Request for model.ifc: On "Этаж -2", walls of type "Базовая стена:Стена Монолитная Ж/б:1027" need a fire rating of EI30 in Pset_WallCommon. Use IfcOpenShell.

First a look at what the model holds.

```python
import ifcopenshell
import ifcopenshell.util.element

model = ifcopenshell.open("model.ifc")
print(model.schema)
storey = next(s for s in model.by_type("IfcBuildingStorey") if s.Name == "Этаж -2")
walls = [e for e in ifcopenshell.util.element.get_decomposition(storey) if e.is_a("IfcWall")]
seen = {}
for e in walls:
    element_type = ifcopenshell.util.element.get_type(e)
    key = (element_type.Name if element_type != e and element_type else None, ifcopenshell.util.element.get_pset(e, "Pset_WallCommon", "FireRating"))
    seen[key] = seen.get(key, 0) + 1
for (name, value), count in sorted(seen.items(), key=str):
    print(count, "x", name, "|", value)
```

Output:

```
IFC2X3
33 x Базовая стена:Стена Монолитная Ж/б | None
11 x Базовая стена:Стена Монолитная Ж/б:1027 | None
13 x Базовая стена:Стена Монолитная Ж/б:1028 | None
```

```python
import ifcopenshell
import ifcopenshell.api.pset
import ifcopenshell.util.element

model = ifcopenshell.open("model.ifc")

storey = next(s for s in model.by_type("IfcBuildingStorey") if s.Name == "Этаж -2")
walls = [e for e in ifcopenshell.util.element.get_decomposition(storey) if e.is_a("IfcWall")]

count = 0
for e in walls:
    element_type = ifcopenshell.util.element.get_type(e)
    if element_type in (None, e) or element_type.Name != "Базовая стена:Стена Монолитная Ж/б:1027":
        continue
    # add_pset returns the element's existing set when there is one.
    pset = ifcopenshell.api.pset.add_pset(model, product=e, name="Pset_WallCommon")
    ifcopenshell.api.pset.edit_pset(model, pset=pset, properties={"FireRating": "EI30"})
    count += 1

print(count, "walls updated")

model.write("model_edited.ifc")
```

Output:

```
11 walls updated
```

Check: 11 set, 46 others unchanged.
